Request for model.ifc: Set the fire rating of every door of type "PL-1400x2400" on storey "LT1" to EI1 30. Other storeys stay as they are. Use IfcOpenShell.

First a look at what the model holds.

```python
import ifcopenshell
import ifcopenshell.util.element

model = ifcopenshell.open("model.ifc")
print(model.schema)
storey = next(s for s in model.by_type("IfcBuildingStorey") if s.Name == "LT1")
doors = [e for e in ifcopenshell.util.element.get_decomposition(storey) if e.is_a("IfcDoor")]
seen = {}
for e in doors:
    element_type = ifcopenshell.util.element.get_type(e)
    key = (element_type.Name if element_type != e and element_type else None, ifcopenshell.util.element.get_pset(e, "Pset_DoorCommon", "FireRating"))
    seen[key] = seen.get(key, 0) + 1
for (name, value), count in sorted(seen.items(), key=str):
    print(count, "x", name, "|", value)
```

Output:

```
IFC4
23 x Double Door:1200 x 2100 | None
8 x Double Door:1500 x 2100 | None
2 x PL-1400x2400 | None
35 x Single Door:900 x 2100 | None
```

```python
import ifcopenshell
import ifcopenshell.api.pset
import ifcopenshell.util.element

model = ifcopenshell.open("model.ifc")

storey = next(s for s in model.by_type("IfcBuildingStorey") if s.Name == "LT1")
doors = [e for e in ifcopenshell.util.element.get_decomposition(storey) if e.is_a("IfcDoor")]

count = 0
for e in doors:
    element_type = ifcopenshell.util.element.get_type(e)
    if element_type in (None, e) or element_type.Name != "PL-1400x2400":
        continue
    # add_pset returns the element's existing set when there is one.
    pset = ifcopenshell.api.pset.add_pset(model, product=e, name="Pset_DoorCommon")
    ifcopenshell.api.pset.edit_pset(model, pset=pset, properties={"FireRating": "EI1 30"})
    count += 1

print(count, "doors updated")

model.write("model_rev.ifc")
```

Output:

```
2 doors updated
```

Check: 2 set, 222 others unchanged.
